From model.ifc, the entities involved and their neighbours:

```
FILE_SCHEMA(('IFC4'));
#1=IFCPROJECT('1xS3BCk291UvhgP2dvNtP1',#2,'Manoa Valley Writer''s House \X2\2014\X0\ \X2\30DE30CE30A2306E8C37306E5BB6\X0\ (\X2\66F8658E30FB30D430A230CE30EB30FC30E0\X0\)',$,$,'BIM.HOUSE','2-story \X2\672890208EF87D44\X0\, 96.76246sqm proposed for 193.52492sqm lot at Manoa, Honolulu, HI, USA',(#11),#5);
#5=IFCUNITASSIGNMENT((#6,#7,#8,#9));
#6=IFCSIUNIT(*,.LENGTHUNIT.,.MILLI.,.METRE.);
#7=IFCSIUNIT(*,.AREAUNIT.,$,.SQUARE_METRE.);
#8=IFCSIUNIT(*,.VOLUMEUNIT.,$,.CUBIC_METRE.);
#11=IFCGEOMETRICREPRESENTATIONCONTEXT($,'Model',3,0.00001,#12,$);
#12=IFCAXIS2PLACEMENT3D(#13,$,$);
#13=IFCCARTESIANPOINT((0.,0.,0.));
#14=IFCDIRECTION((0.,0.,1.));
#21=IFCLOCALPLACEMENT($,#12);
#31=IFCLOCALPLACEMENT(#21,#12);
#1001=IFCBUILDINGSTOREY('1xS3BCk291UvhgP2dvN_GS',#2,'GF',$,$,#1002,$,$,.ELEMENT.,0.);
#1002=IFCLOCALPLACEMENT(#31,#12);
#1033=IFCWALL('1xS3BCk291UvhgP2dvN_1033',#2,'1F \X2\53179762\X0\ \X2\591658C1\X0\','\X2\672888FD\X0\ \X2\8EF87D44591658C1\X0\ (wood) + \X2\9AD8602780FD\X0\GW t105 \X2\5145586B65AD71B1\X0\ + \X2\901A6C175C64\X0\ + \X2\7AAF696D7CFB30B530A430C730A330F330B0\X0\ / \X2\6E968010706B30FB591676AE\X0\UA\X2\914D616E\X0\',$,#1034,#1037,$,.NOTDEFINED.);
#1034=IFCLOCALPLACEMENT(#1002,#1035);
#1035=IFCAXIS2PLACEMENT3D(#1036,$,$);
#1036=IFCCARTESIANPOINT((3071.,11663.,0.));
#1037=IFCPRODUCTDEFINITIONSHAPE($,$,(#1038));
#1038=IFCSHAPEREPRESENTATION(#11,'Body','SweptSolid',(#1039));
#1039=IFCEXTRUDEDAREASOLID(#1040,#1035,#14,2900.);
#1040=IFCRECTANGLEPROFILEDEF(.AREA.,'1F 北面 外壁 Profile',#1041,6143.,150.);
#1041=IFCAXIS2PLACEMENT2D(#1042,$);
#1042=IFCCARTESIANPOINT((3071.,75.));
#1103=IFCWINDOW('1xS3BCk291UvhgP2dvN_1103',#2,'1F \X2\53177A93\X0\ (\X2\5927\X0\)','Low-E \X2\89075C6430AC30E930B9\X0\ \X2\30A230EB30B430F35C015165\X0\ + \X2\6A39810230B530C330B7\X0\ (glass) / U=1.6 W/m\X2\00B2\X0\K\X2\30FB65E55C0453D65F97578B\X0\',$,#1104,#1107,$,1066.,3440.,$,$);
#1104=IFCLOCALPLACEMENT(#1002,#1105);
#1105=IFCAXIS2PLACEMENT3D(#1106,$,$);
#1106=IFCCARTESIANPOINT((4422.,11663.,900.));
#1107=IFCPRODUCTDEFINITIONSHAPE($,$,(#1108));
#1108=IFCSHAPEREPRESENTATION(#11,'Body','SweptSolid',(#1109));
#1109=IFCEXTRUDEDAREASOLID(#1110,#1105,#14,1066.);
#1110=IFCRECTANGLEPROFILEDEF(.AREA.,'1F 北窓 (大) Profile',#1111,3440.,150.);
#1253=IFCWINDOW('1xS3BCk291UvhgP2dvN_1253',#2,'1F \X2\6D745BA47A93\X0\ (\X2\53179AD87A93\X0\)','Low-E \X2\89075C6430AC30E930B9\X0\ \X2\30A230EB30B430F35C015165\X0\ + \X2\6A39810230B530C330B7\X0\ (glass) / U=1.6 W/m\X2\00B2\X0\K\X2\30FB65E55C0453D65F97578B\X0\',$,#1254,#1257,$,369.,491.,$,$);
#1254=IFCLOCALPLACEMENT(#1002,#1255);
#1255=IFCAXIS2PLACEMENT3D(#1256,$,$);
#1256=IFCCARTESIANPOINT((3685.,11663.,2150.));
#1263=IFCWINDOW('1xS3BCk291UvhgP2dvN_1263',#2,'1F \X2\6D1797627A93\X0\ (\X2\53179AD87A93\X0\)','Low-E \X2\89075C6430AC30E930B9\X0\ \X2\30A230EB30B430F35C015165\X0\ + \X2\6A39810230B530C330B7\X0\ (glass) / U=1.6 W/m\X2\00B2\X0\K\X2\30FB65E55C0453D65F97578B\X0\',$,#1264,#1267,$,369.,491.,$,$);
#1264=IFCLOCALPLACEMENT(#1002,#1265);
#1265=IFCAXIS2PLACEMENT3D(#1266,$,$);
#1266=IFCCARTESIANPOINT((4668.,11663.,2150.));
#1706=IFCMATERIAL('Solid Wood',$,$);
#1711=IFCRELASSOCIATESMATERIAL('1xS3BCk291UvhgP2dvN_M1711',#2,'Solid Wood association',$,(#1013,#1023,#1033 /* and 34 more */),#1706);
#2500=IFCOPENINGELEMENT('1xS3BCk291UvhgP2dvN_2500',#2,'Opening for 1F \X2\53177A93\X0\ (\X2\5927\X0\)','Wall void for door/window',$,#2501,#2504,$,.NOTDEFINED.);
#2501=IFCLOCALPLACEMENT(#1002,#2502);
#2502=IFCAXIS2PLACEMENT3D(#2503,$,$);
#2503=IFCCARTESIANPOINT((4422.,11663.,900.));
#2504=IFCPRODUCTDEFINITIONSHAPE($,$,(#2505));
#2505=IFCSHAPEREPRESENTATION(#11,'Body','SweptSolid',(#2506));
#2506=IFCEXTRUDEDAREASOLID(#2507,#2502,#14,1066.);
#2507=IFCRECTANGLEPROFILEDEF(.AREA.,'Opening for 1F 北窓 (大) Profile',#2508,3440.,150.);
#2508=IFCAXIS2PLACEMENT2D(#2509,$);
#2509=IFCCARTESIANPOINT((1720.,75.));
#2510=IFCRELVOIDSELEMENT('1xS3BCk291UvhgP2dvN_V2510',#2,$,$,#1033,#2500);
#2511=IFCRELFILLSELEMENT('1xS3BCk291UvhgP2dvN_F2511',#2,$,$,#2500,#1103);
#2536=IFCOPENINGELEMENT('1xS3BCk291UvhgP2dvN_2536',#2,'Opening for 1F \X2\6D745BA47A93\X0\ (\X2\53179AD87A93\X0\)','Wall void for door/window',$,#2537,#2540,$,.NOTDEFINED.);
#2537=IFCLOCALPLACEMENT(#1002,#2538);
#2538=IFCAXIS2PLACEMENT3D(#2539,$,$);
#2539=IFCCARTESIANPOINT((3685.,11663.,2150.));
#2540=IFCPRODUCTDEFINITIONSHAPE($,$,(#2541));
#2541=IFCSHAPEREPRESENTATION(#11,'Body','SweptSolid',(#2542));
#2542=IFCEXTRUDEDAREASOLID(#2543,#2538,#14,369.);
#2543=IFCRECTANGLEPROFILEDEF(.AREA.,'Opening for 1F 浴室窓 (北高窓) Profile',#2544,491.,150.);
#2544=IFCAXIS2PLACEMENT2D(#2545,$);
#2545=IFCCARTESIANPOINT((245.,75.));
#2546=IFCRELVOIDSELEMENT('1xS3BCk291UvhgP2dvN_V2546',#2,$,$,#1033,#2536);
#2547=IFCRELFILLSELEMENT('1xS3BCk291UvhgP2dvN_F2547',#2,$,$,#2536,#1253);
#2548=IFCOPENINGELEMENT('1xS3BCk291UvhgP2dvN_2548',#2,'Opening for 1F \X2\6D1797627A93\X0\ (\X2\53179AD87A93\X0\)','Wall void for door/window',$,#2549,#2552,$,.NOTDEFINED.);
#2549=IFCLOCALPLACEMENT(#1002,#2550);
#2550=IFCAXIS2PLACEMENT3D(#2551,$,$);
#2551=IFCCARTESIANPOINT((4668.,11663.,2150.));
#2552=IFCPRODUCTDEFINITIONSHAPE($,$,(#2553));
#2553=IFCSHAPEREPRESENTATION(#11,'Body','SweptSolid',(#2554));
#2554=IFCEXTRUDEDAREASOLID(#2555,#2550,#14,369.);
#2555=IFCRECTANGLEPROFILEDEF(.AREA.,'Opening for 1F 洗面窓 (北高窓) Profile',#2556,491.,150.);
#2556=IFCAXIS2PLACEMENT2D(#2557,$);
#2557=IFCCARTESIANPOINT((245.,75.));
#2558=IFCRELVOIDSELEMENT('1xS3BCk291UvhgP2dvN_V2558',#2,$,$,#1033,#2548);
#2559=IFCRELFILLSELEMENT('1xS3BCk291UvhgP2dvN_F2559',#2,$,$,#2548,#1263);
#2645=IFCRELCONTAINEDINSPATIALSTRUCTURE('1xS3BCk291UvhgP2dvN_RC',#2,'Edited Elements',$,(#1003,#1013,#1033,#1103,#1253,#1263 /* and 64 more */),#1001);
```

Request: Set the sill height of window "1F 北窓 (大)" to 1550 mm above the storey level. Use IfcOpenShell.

```python
import numpy as np
import ifcopenshell
import ifcopenshell.api.geometry
import ifcopenshell.geom
import ifcopenshell.util.element
import ifcopenshell.util.placement
import ifcopenshell.util.shape
import ifcopenshell.util.unit

model = ifcopenshell.open("model.ifc")
unit_scale = ifcopenshell.util.unit.calculate_unit_scale(model)

window = model.by_guid("1xS3BCk291UvhgP2dvN_1103")
opening = window.FillsVoids[0].RelatingOpeningElement
storey = ifcopenshell.util.element.get_container(window, ifc_class="IfcBuildingStorey")
level = ifcopenshell.util.placement.get_local_placement(storey.ObjectPlacement)[2, 3]

# The opening's origin need not be at the sill, so measure its lowest point.
shape = ifcopenshell.geom.create_shape(ifcopenshell.geom.settings(), opening)
bottom = ifcopenshell.util.shape.get_shape_bottom_elevation(shape, shape.geometry) / unit_scale
dz = level + 1550.0 - bottom

shift = np.array([0.0, 0.0, dz])
# The window is not placed relative to its opening, so move both.
for product in (opening, window):
    matrix = ifcopenshell.util.placement.get_local_placement(product.ObjectPlacement)
    matrix[:3, 3] += shift
    ifcopenshell.api.geometry.edit_object_placement(model, product=product, matrix=matrix, is_si=False)

print(f"moved by {dz * unit_scale:+.3f} m")

model.write("model_updated.ifc")
```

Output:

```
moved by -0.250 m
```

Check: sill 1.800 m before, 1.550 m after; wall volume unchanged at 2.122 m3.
